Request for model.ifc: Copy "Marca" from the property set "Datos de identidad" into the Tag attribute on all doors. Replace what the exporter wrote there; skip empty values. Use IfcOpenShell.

First a look at what the model holds.

```python
import ifcopenshell
import ifcopenshell.util.element

model = ifcopenshell.open("model.ifc")
print(model.schema)
doors = model.by_type("IfcDoor")
print(len(doors), "doors")
for e in doors[:8]:
    source = ifcopenshell.util.element.get_pset(e, "Datos de identidad", "Marca")
    target = e.Tag
    print(e.id(), repr(source), repr(target), sep=" | ")
```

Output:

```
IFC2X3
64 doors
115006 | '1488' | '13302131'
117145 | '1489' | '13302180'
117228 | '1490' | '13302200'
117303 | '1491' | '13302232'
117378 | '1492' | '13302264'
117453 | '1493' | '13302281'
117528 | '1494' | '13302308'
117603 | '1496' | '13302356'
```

```python
import ifcopenshell
import ifcopenshell.util.element

model = ifcopenshell.open("model.ifc")

count = 0
for e in model.by_type("IfcDoor"):
    value = ifcopenshell.util.element.get_pset(e, "Datos de identidad", "Marca")
    current = e.Tag
    if not value or not value.strip() or current == value:
        continue
    e.Tag = value
    count += 1

print(count, "doors updated")

model.write("model_updated.ifc")
```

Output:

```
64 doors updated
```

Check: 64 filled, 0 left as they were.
